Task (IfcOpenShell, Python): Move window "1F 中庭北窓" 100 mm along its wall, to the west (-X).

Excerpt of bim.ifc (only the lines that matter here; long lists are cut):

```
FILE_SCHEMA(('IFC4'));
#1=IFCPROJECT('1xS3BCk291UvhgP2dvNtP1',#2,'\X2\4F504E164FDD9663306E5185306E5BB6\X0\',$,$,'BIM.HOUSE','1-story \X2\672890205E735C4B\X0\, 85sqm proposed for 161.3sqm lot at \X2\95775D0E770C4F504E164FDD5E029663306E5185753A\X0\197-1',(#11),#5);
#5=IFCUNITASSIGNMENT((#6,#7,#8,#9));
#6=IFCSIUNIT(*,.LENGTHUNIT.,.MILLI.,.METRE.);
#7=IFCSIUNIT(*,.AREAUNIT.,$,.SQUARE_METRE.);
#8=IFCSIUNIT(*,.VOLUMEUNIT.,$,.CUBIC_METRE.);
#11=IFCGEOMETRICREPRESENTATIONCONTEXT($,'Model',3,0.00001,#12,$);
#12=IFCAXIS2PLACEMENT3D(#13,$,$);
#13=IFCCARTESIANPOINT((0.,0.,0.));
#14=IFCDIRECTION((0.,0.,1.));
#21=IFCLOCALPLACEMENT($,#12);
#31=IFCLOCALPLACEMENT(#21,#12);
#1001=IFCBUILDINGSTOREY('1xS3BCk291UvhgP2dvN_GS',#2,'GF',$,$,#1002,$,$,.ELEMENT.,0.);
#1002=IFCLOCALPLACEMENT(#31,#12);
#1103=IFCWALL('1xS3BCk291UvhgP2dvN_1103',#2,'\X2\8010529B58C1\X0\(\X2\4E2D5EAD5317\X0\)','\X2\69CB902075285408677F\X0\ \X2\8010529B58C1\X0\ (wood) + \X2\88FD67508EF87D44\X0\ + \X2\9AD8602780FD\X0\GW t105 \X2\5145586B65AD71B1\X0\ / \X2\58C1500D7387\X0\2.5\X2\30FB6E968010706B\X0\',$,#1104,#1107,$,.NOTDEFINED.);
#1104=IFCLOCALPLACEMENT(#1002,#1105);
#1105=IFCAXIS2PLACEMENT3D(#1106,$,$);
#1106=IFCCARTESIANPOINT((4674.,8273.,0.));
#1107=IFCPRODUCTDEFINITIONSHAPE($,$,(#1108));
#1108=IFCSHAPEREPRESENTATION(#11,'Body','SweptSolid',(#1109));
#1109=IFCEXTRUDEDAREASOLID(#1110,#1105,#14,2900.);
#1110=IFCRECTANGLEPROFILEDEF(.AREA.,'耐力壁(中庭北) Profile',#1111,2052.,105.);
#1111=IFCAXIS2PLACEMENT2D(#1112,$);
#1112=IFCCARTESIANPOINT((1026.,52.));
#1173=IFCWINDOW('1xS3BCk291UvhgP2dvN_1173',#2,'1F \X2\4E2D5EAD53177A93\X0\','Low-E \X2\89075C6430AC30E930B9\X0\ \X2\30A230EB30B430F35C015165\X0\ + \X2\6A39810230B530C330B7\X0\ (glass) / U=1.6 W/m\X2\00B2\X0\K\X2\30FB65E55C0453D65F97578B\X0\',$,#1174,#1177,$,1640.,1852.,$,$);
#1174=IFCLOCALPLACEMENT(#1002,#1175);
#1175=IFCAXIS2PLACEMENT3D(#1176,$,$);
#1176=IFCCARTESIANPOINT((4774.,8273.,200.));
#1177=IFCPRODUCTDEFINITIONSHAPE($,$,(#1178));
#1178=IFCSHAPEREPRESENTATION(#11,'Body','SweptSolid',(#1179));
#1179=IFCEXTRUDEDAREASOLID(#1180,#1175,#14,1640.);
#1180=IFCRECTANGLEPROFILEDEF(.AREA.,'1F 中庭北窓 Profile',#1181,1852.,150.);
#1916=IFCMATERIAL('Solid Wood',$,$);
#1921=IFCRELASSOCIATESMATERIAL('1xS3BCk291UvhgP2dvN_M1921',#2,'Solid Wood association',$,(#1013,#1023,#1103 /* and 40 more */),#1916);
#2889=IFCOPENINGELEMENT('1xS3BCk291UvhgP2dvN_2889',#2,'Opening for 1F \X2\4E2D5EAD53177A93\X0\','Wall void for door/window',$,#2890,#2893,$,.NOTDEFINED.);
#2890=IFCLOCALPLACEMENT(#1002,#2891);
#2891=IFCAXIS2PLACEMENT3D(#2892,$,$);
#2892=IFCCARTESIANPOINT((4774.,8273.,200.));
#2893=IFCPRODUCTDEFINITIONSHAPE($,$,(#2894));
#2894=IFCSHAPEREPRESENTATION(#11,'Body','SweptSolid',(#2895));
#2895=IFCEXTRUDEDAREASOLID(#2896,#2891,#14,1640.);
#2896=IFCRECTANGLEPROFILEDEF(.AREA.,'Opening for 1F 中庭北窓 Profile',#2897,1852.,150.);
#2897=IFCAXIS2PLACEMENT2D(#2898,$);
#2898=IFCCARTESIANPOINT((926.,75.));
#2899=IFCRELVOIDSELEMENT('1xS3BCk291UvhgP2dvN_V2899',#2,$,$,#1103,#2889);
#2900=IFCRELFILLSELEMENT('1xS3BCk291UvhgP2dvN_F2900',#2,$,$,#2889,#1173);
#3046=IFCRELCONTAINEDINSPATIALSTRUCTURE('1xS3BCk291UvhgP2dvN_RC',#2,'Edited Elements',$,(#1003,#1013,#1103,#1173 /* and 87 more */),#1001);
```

```python
import ifcopenshell
import ifcopenshell.api.geometry
import ifcopenshell.util.placement

model = ifcopenshell.open("bim.ifc")

window = model.by_guid("1xS3BCk291UvhgP2dvN_1173")
opening = window.FillsVoids[0].RelatingOpeningElement
wall = opening.VoidsElements[0].RelatingBuildingElement

wall_matrix = ifcopenshell.util.placement.get_local_placement(wall.ObjectPlacement)
shift = wall_matrix[:3, 0] * -100.0
before = ifcopenshell.util.placement.get_local_placement(window.ObjectPlacement)[:3, 3].copy()

# The window is not placed relative to its opening, so move both.
for product in (opening, window):
    matrix = ifcopenshell.util.placement.get_local_placement(product.ObjectPlacement)
    matrix[:3, 3] += shift
    ifcopenshell.api.geometry.edit_object_placement(model, product=product, matrix=matrix, is_si=False)

after = ifcopenshell.util.placement.get_local_placement(window.ObjectPlacement)[:3, 3]
print("window moved by", (after - before).round(3) + 0.0)

model.write("bim_rev.ifc")
```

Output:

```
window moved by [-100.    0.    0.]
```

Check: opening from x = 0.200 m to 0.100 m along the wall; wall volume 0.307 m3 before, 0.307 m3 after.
